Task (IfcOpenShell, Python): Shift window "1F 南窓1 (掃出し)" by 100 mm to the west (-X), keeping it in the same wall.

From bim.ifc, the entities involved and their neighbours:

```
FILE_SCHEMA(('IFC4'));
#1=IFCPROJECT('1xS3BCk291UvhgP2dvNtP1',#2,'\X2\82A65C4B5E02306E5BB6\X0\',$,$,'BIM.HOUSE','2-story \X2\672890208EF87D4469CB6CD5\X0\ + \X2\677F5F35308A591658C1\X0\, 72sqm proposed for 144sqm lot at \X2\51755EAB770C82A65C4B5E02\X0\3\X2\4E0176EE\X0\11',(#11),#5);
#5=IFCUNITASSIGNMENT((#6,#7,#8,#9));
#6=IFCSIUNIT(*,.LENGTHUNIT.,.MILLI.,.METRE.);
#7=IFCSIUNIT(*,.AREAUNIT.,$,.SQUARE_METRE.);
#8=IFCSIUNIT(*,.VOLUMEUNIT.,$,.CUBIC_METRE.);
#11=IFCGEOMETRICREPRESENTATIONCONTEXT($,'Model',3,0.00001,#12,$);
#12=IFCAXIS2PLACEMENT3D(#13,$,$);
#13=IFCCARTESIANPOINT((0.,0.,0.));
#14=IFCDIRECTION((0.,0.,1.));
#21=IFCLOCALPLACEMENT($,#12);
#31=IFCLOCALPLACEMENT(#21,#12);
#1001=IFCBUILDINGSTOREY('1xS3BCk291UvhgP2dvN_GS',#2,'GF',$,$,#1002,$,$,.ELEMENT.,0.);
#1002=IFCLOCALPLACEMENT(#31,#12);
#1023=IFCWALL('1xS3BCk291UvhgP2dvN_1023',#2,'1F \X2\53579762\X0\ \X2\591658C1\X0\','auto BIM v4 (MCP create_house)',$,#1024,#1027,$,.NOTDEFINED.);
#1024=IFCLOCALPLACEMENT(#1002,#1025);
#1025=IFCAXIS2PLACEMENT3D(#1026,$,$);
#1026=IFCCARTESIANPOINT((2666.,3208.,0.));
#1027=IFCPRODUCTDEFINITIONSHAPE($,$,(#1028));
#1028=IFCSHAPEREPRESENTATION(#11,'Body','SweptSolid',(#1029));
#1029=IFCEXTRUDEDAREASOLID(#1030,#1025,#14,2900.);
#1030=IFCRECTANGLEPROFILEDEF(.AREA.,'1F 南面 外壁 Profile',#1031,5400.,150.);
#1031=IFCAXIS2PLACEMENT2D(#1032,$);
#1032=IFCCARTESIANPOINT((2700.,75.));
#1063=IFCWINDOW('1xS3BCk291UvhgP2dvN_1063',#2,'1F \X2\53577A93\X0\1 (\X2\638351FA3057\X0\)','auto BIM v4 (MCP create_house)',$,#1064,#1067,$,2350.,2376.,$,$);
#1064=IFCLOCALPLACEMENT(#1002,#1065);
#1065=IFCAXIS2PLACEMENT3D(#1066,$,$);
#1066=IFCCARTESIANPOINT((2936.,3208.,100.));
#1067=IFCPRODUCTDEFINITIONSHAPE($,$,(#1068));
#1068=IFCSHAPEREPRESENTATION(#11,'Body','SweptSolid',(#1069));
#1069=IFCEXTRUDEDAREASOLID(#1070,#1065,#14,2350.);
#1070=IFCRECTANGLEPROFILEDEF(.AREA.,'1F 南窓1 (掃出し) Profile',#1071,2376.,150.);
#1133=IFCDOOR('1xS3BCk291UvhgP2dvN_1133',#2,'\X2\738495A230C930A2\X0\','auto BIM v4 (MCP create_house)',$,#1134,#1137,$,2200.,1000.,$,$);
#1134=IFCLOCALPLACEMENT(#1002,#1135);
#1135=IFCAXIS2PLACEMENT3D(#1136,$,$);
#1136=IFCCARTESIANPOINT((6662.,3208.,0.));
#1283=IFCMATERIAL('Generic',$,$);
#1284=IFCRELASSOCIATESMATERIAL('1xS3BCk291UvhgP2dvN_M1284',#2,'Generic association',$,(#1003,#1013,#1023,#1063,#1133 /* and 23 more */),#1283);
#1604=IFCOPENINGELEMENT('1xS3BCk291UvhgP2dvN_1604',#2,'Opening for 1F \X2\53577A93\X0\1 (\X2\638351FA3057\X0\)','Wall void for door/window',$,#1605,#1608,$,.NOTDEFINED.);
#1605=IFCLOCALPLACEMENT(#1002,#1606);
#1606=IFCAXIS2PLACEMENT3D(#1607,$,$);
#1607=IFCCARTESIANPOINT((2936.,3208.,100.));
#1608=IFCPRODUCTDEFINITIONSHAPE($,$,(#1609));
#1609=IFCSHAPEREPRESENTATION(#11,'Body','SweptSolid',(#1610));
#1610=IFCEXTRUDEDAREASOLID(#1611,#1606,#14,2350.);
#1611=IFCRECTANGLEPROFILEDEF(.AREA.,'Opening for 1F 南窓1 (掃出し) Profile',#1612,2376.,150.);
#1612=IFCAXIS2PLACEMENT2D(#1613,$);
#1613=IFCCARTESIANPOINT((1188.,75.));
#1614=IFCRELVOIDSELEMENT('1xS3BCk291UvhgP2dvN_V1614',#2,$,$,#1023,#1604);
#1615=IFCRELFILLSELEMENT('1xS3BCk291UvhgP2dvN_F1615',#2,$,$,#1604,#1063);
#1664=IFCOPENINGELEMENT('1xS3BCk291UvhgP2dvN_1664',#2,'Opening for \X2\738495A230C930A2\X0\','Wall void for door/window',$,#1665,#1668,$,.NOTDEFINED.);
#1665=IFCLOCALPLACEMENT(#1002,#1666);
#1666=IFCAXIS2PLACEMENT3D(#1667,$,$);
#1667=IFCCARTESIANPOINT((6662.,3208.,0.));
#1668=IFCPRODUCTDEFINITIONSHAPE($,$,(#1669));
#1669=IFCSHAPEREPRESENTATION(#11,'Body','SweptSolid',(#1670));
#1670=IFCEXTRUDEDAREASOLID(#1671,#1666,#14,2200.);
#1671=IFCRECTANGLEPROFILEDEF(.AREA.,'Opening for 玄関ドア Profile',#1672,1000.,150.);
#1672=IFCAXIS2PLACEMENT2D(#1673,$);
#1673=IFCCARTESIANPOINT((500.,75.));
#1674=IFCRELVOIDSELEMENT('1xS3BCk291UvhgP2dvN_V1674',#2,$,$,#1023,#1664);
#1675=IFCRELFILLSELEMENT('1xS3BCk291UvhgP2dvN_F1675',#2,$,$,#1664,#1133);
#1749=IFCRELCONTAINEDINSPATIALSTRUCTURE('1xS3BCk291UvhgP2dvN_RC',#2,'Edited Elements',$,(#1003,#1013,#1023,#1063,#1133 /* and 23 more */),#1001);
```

```python
import ifcopenshell
import ifcopenshell.api.geometry
import ifcopenshell.util.placement
import ifcopenshell.util.unit

model = ifcopenshell.open("bim.ifc")
unit_scale = ifcopenshell.util.unit.calculate_unit_scale(model)

window = model.by_id(1063)
opening = window.FillsVoids[0].RelatingOpeningElement
wall = opening.VoidsElements[0].RelatingBuildingElement

wall_matrix = ifcopenshell.util.placement.get_local_placement(wall.ObjectPlacement)
shift = wall_matrix[:3, 0] * -0.1 / unit_scale
before = ifcopenshell.util.placement.get_local_placement(window.ObjectPlacement)[:3, 3].copy()

# The window is not placed relative to its opening, so move both.
for product in (opening, window):
    matrix = ifcopenshell.util.placement.get_local_placement(product.ObjectPlacement)
    matrix[:3, 3] += shift
    ifcopenshell.api.geometry.edit_object_placement(model, product=product, matrix=matrix, is_si=False)

after = ifcopenshell.util.placement.get_local_placement(window.ObjectPlacement)[:3, 3]
print("window moved by", (after - before).round(3) + 0.0)

model.write("bim_updated.ifc")
```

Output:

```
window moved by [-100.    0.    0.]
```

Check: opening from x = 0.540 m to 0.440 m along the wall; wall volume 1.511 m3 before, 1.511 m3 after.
